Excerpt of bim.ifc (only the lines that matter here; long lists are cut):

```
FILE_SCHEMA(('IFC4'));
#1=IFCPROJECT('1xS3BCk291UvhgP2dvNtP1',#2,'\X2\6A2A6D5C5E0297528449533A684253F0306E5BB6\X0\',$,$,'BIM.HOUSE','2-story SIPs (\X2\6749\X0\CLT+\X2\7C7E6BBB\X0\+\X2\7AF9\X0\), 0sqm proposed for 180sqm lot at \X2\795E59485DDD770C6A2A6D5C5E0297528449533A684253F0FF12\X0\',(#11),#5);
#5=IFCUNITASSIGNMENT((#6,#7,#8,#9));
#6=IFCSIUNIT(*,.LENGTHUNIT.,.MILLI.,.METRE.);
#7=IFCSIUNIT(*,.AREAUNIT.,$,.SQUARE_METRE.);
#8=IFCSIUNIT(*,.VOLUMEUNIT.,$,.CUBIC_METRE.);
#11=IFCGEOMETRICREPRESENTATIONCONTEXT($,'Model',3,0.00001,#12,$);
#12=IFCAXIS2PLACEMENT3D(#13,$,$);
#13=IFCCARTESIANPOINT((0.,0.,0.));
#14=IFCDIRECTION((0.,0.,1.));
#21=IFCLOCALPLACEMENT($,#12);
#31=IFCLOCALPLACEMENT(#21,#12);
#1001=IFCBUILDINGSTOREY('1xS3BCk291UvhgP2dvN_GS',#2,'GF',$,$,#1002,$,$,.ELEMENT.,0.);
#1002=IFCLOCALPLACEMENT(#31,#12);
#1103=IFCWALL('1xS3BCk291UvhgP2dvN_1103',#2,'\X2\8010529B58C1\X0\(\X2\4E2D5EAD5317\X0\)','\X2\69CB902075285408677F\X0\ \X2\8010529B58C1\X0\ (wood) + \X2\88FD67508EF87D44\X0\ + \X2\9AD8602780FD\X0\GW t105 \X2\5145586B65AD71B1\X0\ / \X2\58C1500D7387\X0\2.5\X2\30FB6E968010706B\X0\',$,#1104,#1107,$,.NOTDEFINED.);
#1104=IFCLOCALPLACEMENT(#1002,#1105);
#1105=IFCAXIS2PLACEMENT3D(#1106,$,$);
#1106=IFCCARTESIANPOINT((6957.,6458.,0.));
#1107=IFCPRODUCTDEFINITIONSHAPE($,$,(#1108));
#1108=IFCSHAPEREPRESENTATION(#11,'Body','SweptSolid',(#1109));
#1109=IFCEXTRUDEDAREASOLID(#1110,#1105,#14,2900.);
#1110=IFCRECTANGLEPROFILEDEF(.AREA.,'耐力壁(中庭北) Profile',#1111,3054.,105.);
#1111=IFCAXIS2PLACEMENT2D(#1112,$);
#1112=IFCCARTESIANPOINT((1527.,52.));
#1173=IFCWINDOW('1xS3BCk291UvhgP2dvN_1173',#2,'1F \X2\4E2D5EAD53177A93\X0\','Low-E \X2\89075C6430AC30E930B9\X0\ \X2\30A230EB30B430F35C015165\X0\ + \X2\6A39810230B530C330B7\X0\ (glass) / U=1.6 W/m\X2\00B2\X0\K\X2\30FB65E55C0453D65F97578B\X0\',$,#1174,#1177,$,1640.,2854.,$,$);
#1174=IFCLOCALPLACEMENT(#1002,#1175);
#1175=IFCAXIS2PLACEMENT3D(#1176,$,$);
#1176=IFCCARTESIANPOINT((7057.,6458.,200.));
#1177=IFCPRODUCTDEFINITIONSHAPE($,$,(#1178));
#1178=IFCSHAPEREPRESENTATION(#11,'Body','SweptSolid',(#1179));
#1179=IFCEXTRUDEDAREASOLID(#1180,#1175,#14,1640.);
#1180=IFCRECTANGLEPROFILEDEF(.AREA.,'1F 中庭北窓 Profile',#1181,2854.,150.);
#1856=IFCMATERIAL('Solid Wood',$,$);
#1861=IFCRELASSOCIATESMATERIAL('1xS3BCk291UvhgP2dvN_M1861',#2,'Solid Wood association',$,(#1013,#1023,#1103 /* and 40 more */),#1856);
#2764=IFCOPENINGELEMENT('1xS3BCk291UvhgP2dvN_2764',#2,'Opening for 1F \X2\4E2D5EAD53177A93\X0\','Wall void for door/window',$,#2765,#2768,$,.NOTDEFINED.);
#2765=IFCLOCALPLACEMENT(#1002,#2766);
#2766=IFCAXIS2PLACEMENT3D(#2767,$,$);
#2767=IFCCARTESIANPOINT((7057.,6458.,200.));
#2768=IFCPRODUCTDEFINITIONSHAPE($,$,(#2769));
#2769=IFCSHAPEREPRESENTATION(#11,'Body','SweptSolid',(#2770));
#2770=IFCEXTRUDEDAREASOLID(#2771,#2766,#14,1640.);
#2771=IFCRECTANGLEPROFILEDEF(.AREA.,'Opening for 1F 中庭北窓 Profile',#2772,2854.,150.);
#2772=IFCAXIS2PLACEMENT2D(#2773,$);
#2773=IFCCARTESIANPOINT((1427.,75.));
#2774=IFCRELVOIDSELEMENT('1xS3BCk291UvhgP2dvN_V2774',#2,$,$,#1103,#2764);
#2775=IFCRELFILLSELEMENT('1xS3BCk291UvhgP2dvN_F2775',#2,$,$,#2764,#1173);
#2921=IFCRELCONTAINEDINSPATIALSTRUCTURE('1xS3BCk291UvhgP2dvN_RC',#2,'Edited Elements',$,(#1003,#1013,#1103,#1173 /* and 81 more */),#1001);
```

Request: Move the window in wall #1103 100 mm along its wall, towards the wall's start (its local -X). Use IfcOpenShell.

```python
import ifcopenshell
import ifcopenshell.api.geometry
import ifcopenshell.util.placement
import ifcopenshell.util.unit

model = ifcopenshell.open("bim.ifc")
unit_scale = ifcopenshell.util.unit.calculate_unit_scale(model)

window = model.by_id(1173)
opening = window.FillsVoids[0].RelatingOpeningElement
wall = opening.VoidsElements[0].RelatingBuildingElement

wall_matrix = ifcopenshell.util.placement.get_local_placement(wall.ObjectPlacement)
shift = wall_matrix[:3, 0] * -0.1 / unit_scale
before = ifcopenshell.util.placement.get_local_placement(window.ObjectPlacement)[:3, 3].copy()

# The window is not placed relative to its opening, so move both.
for product in (opening, window):
    matrix = ifcopenshell.util.placement.get_local_placement(product.ObjectPlacement)
    matrix[:3, 3] += shift
    ifcopenshell.api.geometry.edit_object_placement(model, product=product, matrix=matrix, is_si=False)

after = ifcopenshell.util.placement.get_local_placement(window.ObjectPlacement)[:3, 3]
print("window moved by", (after - before).round(3) + 0.0)

model.write("bim_rev.ifc")
```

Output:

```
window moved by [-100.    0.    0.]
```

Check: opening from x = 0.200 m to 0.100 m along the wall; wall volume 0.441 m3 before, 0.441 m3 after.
